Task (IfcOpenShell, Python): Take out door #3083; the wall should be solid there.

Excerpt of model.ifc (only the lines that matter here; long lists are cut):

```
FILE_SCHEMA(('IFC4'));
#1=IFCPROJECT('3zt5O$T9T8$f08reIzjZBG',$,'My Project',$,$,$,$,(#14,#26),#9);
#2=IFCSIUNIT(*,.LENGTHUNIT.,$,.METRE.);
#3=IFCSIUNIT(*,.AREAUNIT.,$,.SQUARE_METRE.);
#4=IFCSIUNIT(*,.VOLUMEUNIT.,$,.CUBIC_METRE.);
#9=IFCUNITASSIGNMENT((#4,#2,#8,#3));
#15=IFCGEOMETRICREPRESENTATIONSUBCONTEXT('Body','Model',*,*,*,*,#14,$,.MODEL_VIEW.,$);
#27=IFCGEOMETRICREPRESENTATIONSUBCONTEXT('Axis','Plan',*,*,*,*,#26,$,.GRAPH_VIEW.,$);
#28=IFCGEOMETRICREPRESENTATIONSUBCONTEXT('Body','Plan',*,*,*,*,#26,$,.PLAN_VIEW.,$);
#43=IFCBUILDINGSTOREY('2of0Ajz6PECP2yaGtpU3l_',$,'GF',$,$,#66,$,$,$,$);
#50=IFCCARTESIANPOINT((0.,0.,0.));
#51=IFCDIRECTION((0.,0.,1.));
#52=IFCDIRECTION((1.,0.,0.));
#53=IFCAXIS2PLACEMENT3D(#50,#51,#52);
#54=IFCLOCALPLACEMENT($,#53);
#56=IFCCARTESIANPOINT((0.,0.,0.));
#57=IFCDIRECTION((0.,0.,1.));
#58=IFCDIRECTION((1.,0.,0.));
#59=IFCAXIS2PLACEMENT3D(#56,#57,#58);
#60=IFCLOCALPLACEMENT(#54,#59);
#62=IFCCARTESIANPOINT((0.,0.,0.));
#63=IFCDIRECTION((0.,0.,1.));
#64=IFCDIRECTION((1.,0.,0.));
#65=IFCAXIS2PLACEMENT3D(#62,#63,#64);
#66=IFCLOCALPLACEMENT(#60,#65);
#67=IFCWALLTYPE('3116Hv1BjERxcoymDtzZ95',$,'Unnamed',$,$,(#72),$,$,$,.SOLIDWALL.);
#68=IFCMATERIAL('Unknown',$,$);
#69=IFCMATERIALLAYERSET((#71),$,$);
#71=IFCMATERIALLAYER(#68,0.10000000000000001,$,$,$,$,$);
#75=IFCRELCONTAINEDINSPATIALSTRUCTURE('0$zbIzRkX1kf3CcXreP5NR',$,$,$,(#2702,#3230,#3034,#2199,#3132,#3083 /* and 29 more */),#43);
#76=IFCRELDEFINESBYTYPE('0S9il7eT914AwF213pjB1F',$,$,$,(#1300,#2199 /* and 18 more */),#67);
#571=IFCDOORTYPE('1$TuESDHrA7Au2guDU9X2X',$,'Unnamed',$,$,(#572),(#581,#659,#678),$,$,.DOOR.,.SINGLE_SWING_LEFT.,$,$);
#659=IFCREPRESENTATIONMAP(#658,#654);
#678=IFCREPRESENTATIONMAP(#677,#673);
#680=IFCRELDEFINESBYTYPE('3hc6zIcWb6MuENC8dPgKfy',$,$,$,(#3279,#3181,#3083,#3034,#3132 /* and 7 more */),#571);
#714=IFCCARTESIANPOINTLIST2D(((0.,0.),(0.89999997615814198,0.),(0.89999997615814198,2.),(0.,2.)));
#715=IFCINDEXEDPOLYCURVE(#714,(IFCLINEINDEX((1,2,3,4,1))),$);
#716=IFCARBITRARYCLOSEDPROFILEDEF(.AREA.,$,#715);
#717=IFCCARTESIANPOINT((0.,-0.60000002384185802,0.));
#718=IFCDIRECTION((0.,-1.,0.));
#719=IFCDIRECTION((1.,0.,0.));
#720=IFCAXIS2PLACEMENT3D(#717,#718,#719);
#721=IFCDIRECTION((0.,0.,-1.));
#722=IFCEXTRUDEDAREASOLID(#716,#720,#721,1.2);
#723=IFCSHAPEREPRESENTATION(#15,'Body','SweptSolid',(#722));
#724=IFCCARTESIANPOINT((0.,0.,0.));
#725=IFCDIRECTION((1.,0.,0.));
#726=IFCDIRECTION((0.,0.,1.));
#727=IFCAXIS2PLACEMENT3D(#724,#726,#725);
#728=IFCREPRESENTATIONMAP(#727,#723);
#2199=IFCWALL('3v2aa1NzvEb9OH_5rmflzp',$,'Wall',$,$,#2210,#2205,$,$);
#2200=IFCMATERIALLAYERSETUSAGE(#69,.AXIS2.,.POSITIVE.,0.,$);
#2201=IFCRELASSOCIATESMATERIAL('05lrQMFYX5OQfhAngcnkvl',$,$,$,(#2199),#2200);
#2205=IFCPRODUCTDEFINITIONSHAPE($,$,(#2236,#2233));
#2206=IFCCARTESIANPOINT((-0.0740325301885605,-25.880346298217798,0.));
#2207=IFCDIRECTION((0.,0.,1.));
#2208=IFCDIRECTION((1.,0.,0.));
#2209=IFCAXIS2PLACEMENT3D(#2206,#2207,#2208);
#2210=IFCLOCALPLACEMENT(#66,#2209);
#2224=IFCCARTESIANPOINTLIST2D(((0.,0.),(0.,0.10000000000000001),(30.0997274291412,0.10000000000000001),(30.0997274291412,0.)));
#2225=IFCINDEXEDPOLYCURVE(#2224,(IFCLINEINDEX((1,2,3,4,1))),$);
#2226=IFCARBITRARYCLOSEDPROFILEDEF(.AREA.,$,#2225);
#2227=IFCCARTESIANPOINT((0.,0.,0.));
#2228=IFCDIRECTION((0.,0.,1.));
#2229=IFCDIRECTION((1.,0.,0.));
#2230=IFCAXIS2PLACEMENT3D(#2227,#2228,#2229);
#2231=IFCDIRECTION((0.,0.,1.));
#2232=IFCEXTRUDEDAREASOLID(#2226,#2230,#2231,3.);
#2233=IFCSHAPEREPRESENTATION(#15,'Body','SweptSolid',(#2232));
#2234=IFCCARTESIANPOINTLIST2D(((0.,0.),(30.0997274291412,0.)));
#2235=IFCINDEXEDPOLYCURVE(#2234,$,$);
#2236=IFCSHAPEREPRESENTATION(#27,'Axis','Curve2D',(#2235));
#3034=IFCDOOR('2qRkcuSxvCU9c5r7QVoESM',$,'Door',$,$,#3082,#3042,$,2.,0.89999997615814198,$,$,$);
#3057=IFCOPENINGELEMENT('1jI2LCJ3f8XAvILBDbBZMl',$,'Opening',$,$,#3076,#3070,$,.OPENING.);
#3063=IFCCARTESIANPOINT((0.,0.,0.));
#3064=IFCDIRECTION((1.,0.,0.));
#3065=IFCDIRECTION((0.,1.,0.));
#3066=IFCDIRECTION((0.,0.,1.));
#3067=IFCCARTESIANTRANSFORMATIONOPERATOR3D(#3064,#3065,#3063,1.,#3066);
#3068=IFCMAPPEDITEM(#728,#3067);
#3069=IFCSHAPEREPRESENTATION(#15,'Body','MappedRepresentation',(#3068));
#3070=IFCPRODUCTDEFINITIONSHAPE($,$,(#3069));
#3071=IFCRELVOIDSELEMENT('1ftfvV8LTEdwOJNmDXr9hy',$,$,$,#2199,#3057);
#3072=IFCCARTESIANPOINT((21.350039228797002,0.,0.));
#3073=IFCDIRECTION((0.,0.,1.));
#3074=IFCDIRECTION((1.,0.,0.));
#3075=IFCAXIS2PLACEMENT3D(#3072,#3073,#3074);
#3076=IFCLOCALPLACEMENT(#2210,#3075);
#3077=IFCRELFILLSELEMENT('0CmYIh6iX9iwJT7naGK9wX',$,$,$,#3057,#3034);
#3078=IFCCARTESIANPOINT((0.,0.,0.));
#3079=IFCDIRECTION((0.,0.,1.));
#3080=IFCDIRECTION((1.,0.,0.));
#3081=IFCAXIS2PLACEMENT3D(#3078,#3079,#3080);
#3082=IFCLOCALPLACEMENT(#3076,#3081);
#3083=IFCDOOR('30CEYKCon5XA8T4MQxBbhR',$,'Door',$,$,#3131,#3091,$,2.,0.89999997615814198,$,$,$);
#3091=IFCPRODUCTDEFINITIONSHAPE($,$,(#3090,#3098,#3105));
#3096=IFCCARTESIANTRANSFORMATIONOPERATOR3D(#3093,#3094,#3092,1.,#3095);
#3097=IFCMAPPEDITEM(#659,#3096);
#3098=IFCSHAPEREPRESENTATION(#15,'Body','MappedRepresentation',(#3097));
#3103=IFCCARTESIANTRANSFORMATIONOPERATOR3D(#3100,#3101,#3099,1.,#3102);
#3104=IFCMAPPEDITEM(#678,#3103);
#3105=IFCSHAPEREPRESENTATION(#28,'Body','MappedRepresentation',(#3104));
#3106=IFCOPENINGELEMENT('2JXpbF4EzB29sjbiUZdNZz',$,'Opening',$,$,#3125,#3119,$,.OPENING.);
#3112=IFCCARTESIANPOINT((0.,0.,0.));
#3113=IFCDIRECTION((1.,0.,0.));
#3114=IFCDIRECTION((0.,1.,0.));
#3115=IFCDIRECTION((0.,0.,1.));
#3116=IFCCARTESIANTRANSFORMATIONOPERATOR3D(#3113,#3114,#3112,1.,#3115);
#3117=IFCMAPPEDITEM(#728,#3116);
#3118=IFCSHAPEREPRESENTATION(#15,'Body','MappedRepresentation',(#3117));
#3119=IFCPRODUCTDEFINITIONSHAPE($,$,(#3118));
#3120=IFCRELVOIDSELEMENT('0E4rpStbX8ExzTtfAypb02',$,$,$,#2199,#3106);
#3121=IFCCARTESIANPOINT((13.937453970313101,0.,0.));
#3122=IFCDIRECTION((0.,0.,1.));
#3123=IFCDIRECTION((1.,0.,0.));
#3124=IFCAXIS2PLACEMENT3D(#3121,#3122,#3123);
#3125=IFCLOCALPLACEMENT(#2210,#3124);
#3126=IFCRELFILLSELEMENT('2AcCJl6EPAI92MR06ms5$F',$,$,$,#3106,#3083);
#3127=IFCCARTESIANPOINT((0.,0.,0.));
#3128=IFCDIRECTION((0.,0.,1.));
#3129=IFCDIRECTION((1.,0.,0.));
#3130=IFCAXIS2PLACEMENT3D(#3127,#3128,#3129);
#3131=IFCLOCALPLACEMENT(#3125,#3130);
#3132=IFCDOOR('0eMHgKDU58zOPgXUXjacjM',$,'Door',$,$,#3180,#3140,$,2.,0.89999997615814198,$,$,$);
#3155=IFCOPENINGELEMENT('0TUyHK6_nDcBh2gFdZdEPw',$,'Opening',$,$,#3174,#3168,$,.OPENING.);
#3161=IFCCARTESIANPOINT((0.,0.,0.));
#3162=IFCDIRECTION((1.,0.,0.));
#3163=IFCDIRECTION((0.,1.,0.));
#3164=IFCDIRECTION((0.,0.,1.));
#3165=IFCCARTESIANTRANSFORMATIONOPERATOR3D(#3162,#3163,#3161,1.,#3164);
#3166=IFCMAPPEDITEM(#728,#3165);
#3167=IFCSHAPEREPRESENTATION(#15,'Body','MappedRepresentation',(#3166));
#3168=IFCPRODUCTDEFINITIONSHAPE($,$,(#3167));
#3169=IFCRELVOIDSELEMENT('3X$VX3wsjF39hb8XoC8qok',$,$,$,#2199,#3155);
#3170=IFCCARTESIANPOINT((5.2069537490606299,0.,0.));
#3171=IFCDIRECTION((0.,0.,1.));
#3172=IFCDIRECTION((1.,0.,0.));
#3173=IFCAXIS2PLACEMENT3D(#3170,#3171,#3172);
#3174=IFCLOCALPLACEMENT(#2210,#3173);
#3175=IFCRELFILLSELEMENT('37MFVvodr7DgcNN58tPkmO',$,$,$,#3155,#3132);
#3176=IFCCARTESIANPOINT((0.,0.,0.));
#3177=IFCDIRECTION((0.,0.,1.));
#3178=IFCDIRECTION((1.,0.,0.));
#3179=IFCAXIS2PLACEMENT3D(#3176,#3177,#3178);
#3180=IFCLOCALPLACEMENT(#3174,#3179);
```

```python
import ifcopenshell
import ifcopenshell.api.feature
import ifcopenshell.api.root
import ifcopenshell.geom
import ifcopenshell.util.shape

model = ifcopenshell.open("model.ifc")
settings = ifcopenshell.geom.settings()


def volume(element):
    """Net volume in cubic metres, openings subtracted."""
    shape = ifcopenshell.geom.create_shape(settings, element)
    return ifcopenshell.util.shape.get_volume(shape.geometry)


door = model.by_guid("30CEYKCon5XA8T4MQxBbhR")
opening = door.FillsVoids[0].RelatingOpeningElement
wall = opening.VoidsElements[0].RelatingBuildingElement
before = volume(wall)

ifcopenshell.api.root.remove_product(model, product=door)
ifcopenshell.api.feature.remove_feature(model, feature=opening)

after = volume(wall)

print(f"wall volume {before:.3f} -> {after:.3f} m3")

model.write("model_rev.ifc")
```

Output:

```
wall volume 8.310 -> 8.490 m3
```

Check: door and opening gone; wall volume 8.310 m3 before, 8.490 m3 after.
